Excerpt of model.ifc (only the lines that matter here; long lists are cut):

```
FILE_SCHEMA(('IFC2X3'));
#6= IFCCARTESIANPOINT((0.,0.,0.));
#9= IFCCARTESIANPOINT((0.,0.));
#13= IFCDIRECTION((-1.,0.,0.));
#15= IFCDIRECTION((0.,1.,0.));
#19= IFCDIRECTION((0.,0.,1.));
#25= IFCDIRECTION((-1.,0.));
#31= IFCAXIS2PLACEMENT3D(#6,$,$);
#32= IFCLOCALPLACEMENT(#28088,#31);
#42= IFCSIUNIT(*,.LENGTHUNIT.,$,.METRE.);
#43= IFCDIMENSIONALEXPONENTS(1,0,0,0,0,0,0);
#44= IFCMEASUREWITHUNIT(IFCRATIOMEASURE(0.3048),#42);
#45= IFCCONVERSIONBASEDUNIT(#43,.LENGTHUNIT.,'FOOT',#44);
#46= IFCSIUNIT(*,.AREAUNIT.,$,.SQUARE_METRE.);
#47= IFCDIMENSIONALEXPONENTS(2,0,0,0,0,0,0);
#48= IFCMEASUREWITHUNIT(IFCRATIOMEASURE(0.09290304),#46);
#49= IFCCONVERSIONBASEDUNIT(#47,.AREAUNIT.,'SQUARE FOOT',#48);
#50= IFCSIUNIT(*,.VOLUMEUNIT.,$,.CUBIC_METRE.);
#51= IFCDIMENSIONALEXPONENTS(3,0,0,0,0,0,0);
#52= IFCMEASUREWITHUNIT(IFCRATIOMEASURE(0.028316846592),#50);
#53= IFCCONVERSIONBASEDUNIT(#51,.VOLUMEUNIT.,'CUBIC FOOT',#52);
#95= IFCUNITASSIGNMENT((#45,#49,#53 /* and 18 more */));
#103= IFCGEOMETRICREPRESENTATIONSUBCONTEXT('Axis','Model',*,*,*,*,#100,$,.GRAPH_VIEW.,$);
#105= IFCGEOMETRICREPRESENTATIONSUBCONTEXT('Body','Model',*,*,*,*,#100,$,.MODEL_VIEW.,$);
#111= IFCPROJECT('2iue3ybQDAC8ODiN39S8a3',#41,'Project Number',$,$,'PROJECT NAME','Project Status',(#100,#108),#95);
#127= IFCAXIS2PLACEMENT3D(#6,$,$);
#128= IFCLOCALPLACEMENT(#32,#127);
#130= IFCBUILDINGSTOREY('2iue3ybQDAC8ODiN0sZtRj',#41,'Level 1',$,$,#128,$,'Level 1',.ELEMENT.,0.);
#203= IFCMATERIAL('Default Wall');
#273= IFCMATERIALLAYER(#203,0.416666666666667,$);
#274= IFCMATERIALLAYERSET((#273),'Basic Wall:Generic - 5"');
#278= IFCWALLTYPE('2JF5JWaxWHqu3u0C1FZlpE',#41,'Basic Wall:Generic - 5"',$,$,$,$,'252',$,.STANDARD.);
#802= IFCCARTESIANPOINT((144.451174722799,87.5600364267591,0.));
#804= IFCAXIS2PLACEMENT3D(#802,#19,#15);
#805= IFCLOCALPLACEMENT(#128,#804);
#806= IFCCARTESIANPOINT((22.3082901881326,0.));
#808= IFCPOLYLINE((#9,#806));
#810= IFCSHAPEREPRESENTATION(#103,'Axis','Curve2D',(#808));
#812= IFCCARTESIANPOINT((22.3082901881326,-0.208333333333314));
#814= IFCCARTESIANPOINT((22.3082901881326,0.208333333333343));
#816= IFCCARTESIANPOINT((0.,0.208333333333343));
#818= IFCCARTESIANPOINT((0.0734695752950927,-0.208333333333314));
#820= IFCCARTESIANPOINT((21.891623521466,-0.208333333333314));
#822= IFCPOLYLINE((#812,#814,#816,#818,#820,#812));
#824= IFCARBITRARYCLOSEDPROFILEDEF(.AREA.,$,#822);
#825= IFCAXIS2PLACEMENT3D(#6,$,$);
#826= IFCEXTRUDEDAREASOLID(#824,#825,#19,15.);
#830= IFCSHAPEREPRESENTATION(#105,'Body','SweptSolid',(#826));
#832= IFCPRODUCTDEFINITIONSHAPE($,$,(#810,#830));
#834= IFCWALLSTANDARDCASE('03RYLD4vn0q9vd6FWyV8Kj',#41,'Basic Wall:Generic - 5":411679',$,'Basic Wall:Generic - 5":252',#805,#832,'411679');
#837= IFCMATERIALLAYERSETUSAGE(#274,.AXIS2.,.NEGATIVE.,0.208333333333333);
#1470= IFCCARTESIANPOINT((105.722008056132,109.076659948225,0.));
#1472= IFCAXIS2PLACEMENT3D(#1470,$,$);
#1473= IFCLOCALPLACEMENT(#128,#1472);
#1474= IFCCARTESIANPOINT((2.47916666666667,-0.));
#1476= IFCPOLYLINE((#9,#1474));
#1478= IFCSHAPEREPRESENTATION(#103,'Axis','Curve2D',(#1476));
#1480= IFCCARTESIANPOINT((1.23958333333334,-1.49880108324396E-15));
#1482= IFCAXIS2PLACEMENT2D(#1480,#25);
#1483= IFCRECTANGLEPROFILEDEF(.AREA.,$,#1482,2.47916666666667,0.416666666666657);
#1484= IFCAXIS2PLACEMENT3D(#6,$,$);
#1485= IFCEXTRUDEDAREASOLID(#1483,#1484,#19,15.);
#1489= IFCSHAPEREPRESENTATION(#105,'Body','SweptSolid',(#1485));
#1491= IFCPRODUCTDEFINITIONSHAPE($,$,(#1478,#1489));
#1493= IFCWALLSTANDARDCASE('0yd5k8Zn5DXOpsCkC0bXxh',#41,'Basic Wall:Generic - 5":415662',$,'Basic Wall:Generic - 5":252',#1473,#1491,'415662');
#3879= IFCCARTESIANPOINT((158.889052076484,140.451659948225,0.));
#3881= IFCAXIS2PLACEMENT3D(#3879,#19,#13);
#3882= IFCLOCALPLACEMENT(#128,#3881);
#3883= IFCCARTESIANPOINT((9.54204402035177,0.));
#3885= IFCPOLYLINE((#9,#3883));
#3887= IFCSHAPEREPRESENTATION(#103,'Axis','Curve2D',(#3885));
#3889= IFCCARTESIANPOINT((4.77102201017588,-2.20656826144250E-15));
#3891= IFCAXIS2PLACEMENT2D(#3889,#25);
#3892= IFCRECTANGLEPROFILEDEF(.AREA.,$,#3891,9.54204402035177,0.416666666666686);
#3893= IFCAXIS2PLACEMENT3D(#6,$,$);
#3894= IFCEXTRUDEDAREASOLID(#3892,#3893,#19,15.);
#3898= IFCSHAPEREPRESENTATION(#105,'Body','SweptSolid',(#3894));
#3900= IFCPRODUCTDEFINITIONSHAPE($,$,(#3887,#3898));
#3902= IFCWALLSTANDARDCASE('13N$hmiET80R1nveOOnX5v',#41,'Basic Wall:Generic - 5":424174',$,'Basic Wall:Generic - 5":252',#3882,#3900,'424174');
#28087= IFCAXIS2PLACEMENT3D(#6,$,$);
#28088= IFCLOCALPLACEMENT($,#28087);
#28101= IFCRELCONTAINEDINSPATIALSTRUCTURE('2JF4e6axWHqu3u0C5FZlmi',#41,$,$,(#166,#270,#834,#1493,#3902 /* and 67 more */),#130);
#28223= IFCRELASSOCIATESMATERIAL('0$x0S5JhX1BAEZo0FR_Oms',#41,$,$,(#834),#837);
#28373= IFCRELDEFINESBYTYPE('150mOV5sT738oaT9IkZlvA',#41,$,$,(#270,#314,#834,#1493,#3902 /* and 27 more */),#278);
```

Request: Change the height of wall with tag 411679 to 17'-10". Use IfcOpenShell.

```python
import ifcopenshell
import ifcopenshell.geom
import ifcopenshell.util.representation
import ifcopenshell.util.shape
import ifcopenshell.util.unit

model = ifcopenshell.open("model.ifc")
unit_scale = ifcopenshell.util.unit.calculate_unit_scale(model)
settings = ifcopenshell.geom.settings()


def volume(element):
    """Net volume in cubic metres, openings subtracted."""
    shape = ifcopenshell.geom.create_shape(settings, element)
    return ifcopenshell.util.shape.get_volume(shape.geometry)


wall = model.by_guid("03RYLD4vn0q9vd6FWyV8Kj")
before = volume(wall)

body = ifcopenshell.util.representation.get_representation(wall, "Model", "Body")
solid = body.Items[0]
old_height = solid.Depth
solid.Depth = 214 * 0.0254 / unit_scale
after = volume(wall)

print(f"height {old_height:g} -> {solid.Depth:g}, volume {before:.3f} -> {after:.3f} m3")

model.write("model_rev.ifc")
```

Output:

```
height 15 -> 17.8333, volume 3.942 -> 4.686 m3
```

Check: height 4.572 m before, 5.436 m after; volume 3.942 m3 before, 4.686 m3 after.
